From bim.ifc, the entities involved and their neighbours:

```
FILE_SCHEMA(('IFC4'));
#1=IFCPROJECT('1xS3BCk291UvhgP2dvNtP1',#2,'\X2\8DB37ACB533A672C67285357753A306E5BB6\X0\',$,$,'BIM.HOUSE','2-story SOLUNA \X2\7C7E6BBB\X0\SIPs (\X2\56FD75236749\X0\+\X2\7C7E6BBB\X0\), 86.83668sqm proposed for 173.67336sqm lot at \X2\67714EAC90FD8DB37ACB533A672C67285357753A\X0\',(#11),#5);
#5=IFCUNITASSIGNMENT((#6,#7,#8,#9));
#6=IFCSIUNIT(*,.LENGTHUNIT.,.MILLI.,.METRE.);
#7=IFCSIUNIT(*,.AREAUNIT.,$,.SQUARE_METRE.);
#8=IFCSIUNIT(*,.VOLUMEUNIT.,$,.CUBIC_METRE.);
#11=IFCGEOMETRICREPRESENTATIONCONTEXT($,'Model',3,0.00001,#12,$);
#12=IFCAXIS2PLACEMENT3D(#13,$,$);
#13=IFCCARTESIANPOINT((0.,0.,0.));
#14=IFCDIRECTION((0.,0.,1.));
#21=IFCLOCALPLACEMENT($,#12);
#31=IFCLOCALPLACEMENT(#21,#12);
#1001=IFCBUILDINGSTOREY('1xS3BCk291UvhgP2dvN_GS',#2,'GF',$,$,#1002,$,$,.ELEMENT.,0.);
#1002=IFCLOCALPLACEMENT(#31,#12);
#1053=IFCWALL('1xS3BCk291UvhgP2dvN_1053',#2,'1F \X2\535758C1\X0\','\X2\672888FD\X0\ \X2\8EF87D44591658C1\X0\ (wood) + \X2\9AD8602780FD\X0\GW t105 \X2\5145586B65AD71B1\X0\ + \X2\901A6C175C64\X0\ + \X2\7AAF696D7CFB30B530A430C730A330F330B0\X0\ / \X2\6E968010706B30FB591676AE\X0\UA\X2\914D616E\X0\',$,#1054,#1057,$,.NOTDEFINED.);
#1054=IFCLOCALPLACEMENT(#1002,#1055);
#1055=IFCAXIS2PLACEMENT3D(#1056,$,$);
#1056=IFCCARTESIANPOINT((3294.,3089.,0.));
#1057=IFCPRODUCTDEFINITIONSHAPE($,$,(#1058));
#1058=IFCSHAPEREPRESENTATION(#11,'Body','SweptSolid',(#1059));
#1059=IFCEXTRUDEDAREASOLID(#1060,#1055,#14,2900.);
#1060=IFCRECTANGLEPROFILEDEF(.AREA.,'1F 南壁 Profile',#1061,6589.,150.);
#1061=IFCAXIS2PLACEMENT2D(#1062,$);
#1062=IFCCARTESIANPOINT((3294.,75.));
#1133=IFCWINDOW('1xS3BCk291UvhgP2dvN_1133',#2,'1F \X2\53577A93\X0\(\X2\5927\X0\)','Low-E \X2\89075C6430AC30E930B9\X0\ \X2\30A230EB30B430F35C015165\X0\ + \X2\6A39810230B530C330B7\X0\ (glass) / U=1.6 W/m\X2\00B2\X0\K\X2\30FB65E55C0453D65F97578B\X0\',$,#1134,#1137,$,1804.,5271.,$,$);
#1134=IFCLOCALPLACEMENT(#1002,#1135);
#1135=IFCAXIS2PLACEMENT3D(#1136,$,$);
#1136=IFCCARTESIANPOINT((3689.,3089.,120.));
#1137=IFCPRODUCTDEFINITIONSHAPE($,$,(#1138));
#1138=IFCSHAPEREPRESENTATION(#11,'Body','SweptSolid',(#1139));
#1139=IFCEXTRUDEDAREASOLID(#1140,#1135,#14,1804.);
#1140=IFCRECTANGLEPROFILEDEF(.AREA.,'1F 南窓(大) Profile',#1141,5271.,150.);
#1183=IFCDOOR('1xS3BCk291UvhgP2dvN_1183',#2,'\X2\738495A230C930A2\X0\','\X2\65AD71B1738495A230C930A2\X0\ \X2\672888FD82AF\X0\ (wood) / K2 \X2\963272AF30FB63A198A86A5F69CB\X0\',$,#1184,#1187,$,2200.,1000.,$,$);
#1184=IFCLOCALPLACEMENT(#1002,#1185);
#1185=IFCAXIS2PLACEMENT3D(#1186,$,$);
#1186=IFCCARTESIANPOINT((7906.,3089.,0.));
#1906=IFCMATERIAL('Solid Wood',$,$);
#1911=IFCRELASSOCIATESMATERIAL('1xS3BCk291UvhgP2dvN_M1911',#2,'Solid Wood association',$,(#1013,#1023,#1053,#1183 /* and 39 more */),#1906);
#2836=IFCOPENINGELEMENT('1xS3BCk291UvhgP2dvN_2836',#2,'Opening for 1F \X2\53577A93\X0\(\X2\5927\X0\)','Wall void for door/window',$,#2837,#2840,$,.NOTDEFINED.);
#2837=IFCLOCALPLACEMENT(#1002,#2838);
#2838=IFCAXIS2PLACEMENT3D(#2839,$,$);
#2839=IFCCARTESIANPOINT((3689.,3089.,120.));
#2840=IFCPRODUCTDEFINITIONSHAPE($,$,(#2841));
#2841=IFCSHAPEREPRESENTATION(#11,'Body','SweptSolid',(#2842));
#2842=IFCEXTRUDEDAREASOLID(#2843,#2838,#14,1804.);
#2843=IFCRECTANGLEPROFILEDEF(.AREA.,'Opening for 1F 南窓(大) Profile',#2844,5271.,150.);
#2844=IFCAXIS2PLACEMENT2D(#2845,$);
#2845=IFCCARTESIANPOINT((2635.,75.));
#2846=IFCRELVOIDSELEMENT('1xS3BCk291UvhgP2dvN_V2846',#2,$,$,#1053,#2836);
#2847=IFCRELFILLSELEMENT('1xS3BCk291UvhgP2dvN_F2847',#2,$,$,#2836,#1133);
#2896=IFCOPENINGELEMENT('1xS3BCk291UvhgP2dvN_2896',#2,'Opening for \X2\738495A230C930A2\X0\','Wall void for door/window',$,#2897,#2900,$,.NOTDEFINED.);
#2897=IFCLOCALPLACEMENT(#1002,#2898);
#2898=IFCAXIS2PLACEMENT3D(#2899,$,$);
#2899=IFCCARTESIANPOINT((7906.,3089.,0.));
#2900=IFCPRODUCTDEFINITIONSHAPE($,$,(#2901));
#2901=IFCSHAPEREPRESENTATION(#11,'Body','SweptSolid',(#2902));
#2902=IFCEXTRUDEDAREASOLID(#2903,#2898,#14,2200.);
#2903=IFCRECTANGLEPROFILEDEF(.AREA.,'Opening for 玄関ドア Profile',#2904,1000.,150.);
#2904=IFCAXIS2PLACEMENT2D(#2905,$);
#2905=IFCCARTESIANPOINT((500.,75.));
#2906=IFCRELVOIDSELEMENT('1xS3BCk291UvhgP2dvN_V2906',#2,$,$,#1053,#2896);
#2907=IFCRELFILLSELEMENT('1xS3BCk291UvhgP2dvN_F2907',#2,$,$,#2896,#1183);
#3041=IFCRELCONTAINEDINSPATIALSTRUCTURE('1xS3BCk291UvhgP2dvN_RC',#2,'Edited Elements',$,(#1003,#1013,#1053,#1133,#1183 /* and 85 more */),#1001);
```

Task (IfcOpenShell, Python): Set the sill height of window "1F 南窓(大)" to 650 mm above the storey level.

```python
import numpy as np
import ifcopenshell
import ifcopenshell.api.geometry
import ifcopenshell.geom
import ifcopenshell.util.element
import ifcopenshell.util.placement
import ifcopenshell.util.shape
import ifcopenshell.util.unit

model = ifcopenshell.open("bim.ifc")
unit_scale = ifcopenshell.util.unit.calculate_unit_scale(model)

window = model.by_guid("1xS3BCk291UvhgP2dvN_1133")
opening = window.FillsVoids[0].RelatingOpeningElement
storey = ifcopenshell.util.element.get_container(window, ifc_class="IfcBuildingStorey")
level = ifcopenshell.util.placement.get_local_placement(storey.ObjectPlacement)[2, 3]

# The opening's origin need not be at the sill, so measure its lowest point.
shape = ifcopenshell.geom.create_shape(ifcopenshell.geom.settings(), opening)
bottom = ifcopenshell.util.shape.get_shape_bottom_elevation(shape, shape.geometry) / unit_scale
dz = level + 650.0 - bottom

shift = np.array([0.0, 0.0, dz])
# The window is not placed relative to its opening, so move both.
for product in (opening, window):
    matrix = ifcopenshell.util.placement.get_local_placement(product.ObjectPlacement)
    matrix[:3, 3] += shift
    ifcopenshell.api.geometry.edit_object_placement(model, product=product, matrix=matrix, is_si=False)

print(f"moved by {dz * unit_scale:+.3f} m")

model.write("bim-out.ifc")
```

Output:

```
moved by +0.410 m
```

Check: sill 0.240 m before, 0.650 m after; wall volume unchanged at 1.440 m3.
